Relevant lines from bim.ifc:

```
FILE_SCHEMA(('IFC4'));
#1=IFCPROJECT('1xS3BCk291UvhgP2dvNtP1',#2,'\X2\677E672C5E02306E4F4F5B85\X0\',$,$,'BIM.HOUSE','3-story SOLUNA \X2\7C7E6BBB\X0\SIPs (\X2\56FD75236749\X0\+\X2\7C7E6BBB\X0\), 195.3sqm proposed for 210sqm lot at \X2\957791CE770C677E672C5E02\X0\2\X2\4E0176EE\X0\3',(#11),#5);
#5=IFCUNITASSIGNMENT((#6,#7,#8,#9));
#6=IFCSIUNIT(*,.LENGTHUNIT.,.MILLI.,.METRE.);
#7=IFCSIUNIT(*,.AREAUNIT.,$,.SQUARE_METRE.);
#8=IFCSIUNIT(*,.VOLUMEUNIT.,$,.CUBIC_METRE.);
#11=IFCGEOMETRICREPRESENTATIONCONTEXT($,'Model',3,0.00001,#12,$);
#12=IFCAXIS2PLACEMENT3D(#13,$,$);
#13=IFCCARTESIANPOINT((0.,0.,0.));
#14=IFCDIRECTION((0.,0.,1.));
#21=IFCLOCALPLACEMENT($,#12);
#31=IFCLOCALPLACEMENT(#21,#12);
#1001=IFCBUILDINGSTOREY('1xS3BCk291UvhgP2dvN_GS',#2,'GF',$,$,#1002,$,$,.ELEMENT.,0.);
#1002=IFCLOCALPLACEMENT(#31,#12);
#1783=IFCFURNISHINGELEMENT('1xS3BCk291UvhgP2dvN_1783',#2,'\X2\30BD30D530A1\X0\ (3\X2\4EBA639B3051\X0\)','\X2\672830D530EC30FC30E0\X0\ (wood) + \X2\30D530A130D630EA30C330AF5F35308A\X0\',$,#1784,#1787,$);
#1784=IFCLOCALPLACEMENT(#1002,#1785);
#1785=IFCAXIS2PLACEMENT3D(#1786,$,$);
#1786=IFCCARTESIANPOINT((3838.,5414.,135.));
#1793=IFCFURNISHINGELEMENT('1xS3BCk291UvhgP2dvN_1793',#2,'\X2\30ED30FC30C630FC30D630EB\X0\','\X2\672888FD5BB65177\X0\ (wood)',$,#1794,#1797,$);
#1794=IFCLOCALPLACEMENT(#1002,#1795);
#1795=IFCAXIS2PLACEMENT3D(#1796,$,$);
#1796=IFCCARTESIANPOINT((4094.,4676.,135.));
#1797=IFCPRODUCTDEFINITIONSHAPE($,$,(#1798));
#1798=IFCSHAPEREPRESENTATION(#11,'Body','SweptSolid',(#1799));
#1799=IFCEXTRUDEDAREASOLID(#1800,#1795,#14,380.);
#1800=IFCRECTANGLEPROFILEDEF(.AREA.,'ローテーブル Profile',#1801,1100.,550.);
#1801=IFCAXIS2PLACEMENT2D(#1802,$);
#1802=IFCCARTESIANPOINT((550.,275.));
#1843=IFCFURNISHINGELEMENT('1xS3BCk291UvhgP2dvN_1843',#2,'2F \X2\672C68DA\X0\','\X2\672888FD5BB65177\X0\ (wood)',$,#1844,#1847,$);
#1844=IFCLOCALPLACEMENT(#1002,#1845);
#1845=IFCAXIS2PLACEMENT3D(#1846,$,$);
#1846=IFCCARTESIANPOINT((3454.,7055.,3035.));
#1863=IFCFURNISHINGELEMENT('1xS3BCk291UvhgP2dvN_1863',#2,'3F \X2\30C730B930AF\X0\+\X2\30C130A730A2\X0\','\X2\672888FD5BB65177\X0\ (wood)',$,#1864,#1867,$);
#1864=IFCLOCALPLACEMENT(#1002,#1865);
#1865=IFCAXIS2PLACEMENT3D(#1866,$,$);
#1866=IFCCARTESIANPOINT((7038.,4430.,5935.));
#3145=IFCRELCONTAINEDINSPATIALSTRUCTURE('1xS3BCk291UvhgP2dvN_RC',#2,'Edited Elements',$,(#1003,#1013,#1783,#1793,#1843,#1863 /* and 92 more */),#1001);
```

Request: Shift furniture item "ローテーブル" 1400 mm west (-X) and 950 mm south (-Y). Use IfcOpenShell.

```python
import ifcopenshell
import ifcopenshell.api.geometry
import ifcopenshell.util.placement
import ifcopenshell.util.unit

model = ifcopenshell.open("bim.ifc")
unit_scale = ifcopenshell.util.unit.calculate_unit_scale(model)

item = model.by_guid("1xS3BCk291UvhgP2dvN_1793")
matrix = ifcopenshell.util.placement.get_local_placement(item.ObjectPlacement)
matrix[0, 3] -= 1.4 / unit_scale
matrix[1, 3] -= 0.95 / unit_scale
ifcopenshell.api.geometry.edit_object_placement(model, product=item, matrix=matrix, is_si=False)

print(ifcopenshell.util.placement.get_local_placement(item.ObjectPlacement).round(3) + 0.0)

model.write("bim_v2.ifc")
```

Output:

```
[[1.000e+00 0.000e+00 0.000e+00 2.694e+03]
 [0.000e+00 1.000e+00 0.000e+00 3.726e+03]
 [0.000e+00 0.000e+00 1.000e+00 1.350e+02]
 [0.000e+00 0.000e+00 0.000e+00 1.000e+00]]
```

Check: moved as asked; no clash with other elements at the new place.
